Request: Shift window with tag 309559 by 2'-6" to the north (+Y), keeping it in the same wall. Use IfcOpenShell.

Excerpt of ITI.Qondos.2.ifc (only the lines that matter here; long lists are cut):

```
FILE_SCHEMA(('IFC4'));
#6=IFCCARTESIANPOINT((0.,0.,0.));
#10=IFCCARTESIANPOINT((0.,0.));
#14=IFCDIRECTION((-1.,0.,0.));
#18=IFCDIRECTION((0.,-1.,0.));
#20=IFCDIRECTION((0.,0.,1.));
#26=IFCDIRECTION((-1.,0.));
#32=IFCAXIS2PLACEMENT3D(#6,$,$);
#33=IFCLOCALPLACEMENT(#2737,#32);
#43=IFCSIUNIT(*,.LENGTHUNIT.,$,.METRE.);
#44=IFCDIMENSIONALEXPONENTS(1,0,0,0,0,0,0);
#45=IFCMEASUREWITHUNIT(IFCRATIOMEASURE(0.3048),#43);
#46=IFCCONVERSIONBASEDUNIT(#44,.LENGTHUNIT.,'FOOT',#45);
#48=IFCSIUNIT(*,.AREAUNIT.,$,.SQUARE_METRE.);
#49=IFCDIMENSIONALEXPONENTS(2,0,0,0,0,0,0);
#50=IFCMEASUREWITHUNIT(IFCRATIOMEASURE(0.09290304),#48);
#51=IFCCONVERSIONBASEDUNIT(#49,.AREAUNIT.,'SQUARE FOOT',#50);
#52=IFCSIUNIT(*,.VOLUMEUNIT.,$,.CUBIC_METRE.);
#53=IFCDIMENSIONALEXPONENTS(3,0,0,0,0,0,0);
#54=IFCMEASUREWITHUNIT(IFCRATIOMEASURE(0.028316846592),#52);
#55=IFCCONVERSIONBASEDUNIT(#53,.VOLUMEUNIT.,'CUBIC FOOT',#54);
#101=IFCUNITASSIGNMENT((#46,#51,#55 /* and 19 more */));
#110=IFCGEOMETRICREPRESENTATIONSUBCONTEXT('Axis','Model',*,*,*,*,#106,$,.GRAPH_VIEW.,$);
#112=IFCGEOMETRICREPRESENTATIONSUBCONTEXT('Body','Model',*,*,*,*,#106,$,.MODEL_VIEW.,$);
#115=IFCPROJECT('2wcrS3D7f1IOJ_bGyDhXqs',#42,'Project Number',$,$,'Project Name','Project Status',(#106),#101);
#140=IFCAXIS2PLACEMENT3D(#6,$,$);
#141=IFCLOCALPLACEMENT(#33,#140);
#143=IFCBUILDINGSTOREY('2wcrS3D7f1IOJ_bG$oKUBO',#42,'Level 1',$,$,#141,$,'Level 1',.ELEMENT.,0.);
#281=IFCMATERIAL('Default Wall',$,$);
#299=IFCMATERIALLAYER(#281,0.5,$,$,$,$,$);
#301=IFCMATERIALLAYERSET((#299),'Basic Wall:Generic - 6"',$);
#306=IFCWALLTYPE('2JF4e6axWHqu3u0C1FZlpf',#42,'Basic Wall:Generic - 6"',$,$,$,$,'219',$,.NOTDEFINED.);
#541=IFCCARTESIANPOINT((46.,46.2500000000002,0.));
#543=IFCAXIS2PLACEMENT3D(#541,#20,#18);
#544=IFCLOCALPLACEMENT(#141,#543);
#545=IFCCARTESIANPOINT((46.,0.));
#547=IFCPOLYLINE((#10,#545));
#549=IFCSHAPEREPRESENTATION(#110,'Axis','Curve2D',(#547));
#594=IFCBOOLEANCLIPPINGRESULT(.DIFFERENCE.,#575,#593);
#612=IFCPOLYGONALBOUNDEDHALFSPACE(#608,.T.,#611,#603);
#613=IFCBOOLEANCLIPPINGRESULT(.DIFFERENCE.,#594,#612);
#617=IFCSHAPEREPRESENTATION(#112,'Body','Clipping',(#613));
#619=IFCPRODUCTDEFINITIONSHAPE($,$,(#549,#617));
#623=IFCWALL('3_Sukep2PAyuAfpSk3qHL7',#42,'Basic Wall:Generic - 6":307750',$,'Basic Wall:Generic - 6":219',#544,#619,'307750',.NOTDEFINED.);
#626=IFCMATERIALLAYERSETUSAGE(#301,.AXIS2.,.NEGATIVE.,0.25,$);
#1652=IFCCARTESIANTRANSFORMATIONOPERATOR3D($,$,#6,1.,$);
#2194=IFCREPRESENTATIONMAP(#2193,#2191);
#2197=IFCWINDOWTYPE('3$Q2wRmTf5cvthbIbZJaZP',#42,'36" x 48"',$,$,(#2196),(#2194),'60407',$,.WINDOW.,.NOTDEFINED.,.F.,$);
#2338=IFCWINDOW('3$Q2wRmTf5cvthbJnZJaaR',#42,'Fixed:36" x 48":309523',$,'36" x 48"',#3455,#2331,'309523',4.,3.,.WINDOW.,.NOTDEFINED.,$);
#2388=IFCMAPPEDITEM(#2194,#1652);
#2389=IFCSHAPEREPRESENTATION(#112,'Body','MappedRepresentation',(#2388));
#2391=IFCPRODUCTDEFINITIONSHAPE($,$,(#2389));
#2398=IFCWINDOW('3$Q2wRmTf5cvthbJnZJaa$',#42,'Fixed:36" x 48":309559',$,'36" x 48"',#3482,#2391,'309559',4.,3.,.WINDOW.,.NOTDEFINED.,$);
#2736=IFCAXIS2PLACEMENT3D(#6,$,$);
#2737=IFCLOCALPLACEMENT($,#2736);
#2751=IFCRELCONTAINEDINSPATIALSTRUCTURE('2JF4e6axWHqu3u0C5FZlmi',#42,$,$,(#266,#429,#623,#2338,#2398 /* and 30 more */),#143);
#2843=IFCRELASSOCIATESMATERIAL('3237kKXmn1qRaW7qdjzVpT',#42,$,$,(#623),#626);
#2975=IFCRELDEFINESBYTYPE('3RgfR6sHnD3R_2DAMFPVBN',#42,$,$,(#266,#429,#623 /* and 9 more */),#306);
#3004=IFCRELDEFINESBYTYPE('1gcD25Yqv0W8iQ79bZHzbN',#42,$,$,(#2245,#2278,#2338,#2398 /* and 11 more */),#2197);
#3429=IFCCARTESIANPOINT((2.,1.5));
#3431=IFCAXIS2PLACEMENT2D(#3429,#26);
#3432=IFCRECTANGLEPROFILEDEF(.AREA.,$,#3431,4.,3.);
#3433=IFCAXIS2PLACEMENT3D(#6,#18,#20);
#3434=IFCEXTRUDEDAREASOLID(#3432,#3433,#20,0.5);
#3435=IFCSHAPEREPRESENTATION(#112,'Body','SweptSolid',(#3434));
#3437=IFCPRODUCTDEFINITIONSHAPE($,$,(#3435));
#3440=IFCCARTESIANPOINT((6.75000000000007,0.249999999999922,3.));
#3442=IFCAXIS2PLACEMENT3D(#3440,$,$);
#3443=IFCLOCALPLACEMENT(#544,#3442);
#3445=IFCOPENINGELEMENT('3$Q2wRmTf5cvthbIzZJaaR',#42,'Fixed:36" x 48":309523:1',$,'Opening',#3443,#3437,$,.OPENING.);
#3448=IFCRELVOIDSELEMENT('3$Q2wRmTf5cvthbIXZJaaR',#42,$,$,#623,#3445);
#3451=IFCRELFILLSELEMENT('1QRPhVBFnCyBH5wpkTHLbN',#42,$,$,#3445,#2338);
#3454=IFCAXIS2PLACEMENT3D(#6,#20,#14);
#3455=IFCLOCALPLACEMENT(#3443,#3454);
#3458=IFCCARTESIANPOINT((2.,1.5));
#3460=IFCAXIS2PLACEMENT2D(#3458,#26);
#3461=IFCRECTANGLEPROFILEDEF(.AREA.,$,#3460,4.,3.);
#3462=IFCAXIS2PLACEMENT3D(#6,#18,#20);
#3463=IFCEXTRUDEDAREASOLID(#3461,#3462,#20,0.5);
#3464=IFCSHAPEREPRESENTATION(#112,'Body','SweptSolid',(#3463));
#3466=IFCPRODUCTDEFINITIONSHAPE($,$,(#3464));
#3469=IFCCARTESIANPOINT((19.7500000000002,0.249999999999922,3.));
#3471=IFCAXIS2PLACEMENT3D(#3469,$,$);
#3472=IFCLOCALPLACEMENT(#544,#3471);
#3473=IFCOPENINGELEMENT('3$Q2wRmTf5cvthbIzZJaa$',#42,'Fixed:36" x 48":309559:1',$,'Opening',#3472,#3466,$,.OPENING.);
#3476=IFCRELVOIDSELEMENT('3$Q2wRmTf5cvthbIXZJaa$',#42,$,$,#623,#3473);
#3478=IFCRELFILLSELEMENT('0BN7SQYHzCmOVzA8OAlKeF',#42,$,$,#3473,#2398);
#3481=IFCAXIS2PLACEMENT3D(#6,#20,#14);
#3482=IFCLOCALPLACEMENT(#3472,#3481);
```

```python
import ifcopenshell
import ifcopenshell.api.geometry
import ifcopenshell.util.placement
import ifcopenshell.util.unit

model = ifcopenshell.open("ITI.Qondos.2.ifc")
unit_scale = ifcopenshell.util.unit.calculate_unit_scale(model)

window = model.by_id(2398)
opening = window.FillsVoids[0].RelatingOpeningElement
wall = opening.VoidsElements[0].RelatingBuildingElement

wall_matrix = ifcopenshell.util.placement.get_local_placement(wall.ObjectPlacement)
shift = wall_matrix[:3, 0] * -30 * 0.0254 / unit_scale
before = ifcopenshell.util.placement.get_local_placement(window.ObjectPlacement)[:3, 3].copy()

# The window is placed relative to its opening, so it follows when the opening moves.
matrix = ifcopenshell.util.placement.get_local_placement(opening.ObjectPlacement)
matrix[:3, 3] += shift
ifcopenshell.api.geometry.edit_object_placement(
    model, product=opening, matrix=matrix, is_si=False, should_transform_children=True
)

after = ifcopenshell.util.placement.get_local_placement(window.ObjectPlacement)[:3, 3]
print("window moved by", (after - before).round(3) + 0.0)

model.write("ITI.Qondos.2_edited.ifc")
```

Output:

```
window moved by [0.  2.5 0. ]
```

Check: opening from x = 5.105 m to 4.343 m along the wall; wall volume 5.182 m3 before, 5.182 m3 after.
